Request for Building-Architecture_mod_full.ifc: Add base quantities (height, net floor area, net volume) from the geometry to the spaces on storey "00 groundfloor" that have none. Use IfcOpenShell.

First a look at what the model holds.

```python
import ifcopenshell
import ifcopenshell.util.element
import ifcopenshell.util.unit

model = ifcopenshell.open("Building-Architecture_mod_full.ifc")
print(model.schema)
for unit_type in ("LENGTHUNIT", "AREAUNIT", "VOLUMEUNIT"):
    print(unit_type, ifcopenshell.util.unit.calculate_unit_scale(model, unit_type))
storey = next(s for s in model.by_type("IfcBuildingStorey") if s.Name == "00 groundfloor")
spaces = [e for e in ifcopenshell.util.element.get_decomposition(storey) if e.is_a("IfcSpace")]
for e in sorted(spaces, key=lambda e: e.id()):
    print(e.id(), e.is_a(), e.Name, list(ifcopenshell.util.element.get_psets(e, qtos_only=True)), sep=" | ")
```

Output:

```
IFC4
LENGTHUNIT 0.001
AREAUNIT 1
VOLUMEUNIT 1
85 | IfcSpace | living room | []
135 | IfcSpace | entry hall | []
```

```python
import ifcopenshell
import ifcopenshell.api.pset
import ifcopenshell.geom
import ifcopenshell.util.element
import ifcopenshell.util.shape
import ifcopenshell.util.unit

model = ifcopenshell.open("Building-Architecture_mod_full.ifc")
unit_scale = ifcopenshell.util.unit.calculate_unit_scale(model)
area_scale = ifcopenshell.util.unit.calculate_unit_scale(model, "AREAUNIT")
volume_scale = ifcopenshell.util.unit.calculate_unit_scale(model, "VOLUMEUNIT")
settings = ifcopenshell.geom.settings()

storey = next(s for s in model.by_type("IfcBuildingStorey") if s.Name == "00 groundfloor")
spaces = [e for e in ifcopenshell.util.element.get_decomposition(storey) if e.is_a("IfcSpace")]

for e in sorted(spaces, key=lambda e: e.id()):
    if ifcopenshell.util.element.get_psets(e, qtos_only=True, should_inherit=False):
        continue
    # Geometry comes back in metres, in the element's own axes.
    shape = ifcopenshell.geom.create_shape(settings, e)
    values = {
        "Height": ifcopenshell.util.shape.get_z(shape.geometry) / unit_scale,
        "NetFloorArea": ifcopenshell.util.shape.get_footprint_area(shape.geometry) / area_scale,
        "NetVolume": ifcopenshell.util.shape.get_volume(shape.geometry) / volume_scale,
    }
    qto = ifcopenshell.api.pset.add_qto(model, product=e, name="Qto_SpaceBaseQuantities")
    ifcopenshell.api.pset.edit_qto(model, qto=qto, properties=values)
    print(e.id(), {k: round(v, 3) for k, v in values.items()})

model.write("Building-Architecture_mod_full_updated.ifc")
```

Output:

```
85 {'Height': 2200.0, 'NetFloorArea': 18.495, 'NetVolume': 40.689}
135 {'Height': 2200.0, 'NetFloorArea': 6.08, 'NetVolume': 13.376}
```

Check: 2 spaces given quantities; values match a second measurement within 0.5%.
